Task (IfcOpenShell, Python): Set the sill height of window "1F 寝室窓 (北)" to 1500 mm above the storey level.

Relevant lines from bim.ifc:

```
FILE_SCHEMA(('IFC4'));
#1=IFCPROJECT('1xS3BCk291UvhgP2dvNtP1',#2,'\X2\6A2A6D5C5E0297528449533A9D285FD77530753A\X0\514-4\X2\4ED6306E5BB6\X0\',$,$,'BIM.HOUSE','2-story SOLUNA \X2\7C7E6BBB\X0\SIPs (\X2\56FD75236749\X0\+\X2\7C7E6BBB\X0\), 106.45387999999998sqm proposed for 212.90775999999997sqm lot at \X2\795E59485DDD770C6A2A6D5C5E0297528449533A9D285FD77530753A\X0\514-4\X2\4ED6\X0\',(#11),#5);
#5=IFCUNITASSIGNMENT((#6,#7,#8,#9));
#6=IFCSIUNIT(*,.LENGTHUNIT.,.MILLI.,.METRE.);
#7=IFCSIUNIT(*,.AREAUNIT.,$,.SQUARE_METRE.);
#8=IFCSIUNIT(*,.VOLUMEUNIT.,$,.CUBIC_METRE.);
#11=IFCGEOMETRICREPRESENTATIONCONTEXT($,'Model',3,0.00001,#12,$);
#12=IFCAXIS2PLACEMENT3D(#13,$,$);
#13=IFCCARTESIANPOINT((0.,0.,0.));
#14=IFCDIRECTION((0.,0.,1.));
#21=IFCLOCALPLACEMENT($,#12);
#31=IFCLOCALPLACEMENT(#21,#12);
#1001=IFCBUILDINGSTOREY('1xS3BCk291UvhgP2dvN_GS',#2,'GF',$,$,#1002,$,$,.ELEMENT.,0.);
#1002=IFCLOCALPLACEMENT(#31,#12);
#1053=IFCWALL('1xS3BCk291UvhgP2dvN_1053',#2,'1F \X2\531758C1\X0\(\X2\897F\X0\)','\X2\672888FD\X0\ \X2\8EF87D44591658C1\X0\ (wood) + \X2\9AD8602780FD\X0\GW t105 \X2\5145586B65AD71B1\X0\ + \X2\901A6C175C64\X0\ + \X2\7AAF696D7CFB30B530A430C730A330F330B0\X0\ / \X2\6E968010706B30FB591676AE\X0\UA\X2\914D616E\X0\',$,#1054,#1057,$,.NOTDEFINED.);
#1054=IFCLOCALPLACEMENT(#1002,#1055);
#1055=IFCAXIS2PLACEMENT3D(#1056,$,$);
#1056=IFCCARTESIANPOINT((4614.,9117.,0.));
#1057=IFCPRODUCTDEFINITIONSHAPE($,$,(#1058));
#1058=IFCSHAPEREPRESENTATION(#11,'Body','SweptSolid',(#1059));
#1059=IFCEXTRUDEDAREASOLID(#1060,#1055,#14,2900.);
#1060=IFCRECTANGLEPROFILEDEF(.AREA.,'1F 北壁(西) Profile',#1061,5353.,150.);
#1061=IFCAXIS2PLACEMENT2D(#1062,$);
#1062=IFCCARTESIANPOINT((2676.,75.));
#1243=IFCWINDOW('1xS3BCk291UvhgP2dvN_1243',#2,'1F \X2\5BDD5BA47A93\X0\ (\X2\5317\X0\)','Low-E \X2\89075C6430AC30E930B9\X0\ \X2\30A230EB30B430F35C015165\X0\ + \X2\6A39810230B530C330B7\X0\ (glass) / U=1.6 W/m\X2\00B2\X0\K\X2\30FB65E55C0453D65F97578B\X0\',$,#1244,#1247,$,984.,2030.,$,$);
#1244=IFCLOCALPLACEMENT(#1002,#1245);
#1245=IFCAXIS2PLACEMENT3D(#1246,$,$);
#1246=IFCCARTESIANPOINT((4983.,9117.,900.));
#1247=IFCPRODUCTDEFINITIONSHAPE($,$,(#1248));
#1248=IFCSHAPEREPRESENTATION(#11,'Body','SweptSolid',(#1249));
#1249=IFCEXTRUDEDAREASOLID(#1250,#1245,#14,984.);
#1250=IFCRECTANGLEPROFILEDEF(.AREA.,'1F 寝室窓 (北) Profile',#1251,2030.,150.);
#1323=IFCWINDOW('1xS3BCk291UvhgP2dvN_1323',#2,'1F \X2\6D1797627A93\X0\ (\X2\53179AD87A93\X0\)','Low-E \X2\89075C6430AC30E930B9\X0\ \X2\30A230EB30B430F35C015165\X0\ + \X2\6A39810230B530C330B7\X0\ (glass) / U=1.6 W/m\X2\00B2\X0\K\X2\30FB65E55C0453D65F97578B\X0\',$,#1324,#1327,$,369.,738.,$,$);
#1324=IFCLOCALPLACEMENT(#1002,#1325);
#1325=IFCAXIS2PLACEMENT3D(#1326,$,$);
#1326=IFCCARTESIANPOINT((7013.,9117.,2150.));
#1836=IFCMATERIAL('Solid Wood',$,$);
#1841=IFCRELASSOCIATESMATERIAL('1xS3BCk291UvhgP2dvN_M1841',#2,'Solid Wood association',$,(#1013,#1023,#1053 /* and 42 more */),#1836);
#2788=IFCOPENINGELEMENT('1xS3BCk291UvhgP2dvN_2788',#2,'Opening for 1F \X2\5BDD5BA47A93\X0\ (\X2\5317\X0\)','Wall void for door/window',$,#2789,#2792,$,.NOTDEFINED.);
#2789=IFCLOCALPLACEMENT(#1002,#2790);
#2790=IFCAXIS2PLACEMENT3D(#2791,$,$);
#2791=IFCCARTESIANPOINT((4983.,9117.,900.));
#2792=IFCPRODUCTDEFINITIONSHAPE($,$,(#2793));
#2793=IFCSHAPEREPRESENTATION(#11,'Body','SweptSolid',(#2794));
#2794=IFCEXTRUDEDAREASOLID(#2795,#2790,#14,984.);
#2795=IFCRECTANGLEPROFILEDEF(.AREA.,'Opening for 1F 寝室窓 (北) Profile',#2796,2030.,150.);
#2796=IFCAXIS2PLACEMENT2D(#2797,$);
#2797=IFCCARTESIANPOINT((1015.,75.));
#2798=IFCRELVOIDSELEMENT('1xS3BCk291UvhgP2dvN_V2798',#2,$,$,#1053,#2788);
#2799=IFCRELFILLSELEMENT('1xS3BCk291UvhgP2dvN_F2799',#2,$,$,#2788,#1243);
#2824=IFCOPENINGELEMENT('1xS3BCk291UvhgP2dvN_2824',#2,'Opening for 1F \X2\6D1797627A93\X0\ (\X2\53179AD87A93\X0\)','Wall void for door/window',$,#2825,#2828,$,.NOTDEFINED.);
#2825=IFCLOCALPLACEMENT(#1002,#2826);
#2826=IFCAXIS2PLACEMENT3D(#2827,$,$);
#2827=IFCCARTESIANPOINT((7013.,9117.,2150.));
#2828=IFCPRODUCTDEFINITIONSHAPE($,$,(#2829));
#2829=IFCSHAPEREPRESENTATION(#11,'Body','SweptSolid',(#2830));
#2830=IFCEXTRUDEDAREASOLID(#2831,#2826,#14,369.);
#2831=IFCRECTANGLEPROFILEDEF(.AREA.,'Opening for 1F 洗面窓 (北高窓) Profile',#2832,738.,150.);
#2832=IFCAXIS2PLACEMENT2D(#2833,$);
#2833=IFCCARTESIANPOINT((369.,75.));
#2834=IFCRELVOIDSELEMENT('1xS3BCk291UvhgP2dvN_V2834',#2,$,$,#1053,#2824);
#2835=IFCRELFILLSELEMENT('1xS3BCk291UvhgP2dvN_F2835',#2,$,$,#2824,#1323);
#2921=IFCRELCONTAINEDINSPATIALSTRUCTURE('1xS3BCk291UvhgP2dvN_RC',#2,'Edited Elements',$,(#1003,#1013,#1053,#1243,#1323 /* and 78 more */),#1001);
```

```python
import numpy as np
import ifcopenshell
import ifcopenshell.api.geometry
import ifcopenshell.geom
import ifcopenshell.util.element
import ifcopenshell.util.placement
import ifcopenshell.util.shape
import ifcopenshell.util.unit

model = ifcopenshell.open("bim.ifc")
unit_scale = ifcopenshell.util.unit.calculate_unit_scale(model)

window = model.by_id(1243)
opening = window.FillsVoids[0].RelatingOpeningElement
storey = ifcopenshell.util.element.get_container(window, ifc_class="IfcBuildingStorey")
level = ifcopenshell.util.placement.get_local_placement(storey.ObjectPlacement)[2, 3]

# The opening's origin need not be at the sill, so measure its lowest point.
shape = ifcopenshell.geom.create_shape(ifcopenshell.geom.settings(), opening)
bottom = ifcopenshell.util.shape.get_shape_bottom_elevation(shape, shape.geometry) / unit_scale
dz = level + 1.5 / unit_scale - bottom

shift = np.array([0.0, 0.0, dz])
# The window is not placed relative to its opening, so move both.
for product in (opening, window):
    matrix = ifcopenshell.util.placement.get_local_placement(product.ObjectPlacement)
    matrix[:3, 3] += shift
    ifcopenshell.api.geometry.edit_object_placement(model, product=product, matrix=matrix, is_si=False)

print(f"moved by {dz * unit_scale:+.3f} m")

model.write("bim_edited.ifc")
```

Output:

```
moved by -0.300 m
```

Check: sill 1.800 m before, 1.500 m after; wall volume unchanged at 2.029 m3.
